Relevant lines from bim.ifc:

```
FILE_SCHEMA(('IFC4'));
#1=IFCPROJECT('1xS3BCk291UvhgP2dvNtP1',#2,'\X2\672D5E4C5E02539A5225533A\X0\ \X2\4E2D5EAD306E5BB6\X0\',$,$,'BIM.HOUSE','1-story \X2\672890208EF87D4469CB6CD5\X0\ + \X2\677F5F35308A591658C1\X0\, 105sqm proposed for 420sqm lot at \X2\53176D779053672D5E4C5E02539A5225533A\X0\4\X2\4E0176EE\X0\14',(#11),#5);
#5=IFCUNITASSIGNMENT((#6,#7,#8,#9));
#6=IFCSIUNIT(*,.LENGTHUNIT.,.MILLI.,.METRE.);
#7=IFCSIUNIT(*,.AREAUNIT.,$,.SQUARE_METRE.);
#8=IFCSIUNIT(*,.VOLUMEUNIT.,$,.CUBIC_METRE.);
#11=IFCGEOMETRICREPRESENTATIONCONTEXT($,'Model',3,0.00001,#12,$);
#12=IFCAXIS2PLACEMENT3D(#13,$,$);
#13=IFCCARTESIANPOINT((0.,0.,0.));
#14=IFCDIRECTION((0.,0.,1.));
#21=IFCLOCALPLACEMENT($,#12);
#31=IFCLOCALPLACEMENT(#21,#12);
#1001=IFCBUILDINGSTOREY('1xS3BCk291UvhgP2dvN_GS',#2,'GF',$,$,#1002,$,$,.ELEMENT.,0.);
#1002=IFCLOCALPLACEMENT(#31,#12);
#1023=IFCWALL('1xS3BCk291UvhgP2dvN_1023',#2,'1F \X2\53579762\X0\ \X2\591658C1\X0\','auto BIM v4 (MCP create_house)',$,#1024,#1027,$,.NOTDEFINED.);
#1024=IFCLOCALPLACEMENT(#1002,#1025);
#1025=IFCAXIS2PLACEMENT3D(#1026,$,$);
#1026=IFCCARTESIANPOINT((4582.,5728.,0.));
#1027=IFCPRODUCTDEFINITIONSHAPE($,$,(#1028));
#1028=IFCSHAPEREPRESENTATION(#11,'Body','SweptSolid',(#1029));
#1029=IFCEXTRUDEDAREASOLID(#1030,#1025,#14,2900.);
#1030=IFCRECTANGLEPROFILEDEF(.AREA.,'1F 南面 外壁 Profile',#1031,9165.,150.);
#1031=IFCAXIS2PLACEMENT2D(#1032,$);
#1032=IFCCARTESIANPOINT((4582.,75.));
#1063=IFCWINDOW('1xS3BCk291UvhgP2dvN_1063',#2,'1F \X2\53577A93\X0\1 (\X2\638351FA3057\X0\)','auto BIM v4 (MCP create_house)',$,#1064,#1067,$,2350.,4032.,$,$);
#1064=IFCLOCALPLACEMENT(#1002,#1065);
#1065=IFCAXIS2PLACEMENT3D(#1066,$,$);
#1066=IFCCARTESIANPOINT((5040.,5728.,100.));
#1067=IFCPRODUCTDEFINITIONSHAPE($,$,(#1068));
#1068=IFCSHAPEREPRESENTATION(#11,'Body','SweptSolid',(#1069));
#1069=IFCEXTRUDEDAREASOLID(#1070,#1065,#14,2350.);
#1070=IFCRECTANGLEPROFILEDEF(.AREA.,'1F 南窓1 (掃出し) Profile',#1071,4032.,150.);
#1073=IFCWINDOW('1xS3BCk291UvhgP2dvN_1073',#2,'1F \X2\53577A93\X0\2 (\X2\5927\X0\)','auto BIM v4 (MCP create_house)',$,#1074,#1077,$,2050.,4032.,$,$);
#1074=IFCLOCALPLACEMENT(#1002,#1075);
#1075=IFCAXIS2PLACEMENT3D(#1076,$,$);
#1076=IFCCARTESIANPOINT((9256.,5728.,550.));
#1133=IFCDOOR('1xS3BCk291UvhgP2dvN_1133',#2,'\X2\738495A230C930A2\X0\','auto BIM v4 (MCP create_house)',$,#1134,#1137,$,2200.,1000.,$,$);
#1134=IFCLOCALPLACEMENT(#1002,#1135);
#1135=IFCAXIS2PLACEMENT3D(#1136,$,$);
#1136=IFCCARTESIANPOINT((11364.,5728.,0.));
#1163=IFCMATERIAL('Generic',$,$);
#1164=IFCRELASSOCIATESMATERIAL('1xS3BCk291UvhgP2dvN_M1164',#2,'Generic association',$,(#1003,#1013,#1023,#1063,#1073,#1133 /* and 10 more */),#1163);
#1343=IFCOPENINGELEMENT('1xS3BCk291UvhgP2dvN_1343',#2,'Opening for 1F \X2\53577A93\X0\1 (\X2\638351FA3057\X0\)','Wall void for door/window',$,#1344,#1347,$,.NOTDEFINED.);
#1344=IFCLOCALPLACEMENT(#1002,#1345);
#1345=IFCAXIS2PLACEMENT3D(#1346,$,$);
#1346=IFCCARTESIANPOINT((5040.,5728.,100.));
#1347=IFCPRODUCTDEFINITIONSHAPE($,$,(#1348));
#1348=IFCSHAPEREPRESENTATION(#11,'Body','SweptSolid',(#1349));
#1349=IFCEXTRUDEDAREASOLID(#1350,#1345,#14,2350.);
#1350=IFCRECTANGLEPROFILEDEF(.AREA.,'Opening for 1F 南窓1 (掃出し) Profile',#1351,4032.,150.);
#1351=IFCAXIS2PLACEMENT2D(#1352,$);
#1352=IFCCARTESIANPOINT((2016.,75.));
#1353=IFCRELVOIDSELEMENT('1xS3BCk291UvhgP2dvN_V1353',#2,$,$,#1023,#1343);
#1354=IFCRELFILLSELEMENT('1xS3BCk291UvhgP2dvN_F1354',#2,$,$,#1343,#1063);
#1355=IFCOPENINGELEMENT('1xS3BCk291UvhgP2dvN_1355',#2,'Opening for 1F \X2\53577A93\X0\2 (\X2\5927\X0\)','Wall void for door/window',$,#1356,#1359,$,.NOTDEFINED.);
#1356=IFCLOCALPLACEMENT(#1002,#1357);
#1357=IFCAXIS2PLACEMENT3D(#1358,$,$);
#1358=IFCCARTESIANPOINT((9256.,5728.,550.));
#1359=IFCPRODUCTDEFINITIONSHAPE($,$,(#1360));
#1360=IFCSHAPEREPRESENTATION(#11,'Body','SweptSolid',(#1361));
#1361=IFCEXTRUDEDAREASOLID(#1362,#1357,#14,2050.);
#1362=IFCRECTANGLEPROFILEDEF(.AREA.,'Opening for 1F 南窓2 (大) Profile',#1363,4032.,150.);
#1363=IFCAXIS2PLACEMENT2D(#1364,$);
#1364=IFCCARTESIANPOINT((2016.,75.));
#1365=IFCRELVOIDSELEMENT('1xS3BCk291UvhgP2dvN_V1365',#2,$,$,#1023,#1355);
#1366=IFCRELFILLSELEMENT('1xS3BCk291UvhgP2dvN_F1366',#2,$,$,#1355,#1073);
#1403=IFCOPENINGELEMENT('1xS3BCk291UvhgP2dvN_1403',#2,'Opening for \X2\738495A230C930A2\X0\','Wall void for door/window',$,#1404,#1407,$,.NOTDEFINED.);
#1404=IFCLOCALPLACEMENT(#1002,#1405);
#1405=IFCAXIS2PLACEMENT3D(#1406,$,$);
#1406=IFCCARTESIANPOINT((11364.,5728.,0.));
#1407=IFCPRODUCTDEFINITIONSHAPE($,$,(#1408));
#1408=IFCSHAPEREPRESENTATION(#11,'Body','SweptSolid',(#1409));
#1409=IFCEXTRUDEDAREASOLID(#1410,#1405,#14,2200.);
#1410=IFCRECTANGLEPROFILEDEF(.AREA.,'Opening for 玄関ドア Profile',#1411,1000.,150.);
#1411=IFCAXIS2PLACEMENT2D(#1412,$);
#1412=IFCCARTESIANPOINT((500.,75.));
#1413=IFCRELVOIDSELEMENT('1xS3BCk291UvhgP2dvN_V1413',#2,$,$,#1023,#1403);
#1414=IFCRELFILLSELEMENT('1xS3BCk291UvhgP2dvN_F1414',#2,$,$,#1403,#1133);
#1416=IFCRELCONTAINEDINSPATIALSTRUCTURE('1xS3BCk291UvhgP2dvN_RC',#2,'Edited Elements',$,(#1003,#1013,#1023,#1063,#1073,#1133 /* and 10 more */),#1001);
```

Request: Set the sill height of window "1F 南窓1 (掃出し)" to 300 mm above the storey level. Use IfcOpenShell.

```python
import numpy as np
import ifcopenshell
import ifcopenshell.api.geometry
import ifcopenshell.geom
import ifcopenshell.util.element
import ifcopenshell.util.placement
import ifcopenshell.util.shape
import ifcopenshell.util.unit

model = ifcopenshell.open("bim.ifc")
unit_scale = ifcopenshell.util.unit.calculate_unit_scale(model)

window = model.by_guid("1xS3BCk291UvhgP2dvN_1063")
opening = window.FillsVoids[0].RelatingOpeningElement
storey = ifcopenshell.util.element.get_container(window, ifc_class="IfcBuildingStorey")
level = ifcopenshell.util.placement.get_local_placement(storey.ObjectPlacement)[2, 3]

# The opening's origin need not be at the sill, so measure its lowest point.
shape = ifcopenshell.geom.create_shape(ifcopenshell.geom.settings(), opening)
bottom = ifcopenshell.util.shape.get_shape_bottom_elevation(shape, shape.geometry) / unit_scale
dz = level + 300.0 - bottom

shift = np.array([0.0, 0.0, dz])
# The window is not placed relative to its opening, so move both.
for product in (opening, window):
    matrix = ifcopenshell.util.placement.get_local_placement(product.ObjectPlacement)
    matrix[:3, 3] += shift
    ifcopenshell.api.geometry.edit_object_placement(model, product=product, matrix=matrix, is_si=False)

print(f"moved by {dz * unit_scale:+.3f} m")

model.write("bim_v2.ifc")
```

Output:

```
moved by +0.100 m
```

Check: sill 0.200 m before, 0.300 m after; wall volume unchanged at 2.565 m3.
